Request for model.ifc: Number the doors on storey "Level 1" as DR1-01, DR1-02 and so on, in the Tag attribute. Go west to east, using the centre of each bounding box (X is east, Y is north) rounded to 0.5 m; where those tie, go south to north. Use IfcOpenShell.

First a look at what the model holds.

```python
import ifcopenshell
import ifcopenshell.util.element
import ifcopenshell.util.placement

model = ifcopenshell.open("model.ifc")
print(model.schema)
storey = next(s for s in model.by_type("IfcBuildingStorey") if s.Name == "Level 1")
doors = [e for e in ifcopenshell.util.element.get_decomposition(storey) if e.is_a("IfcDoor")]
for e in sorted(doors, key=lambda e: e.id()):
    origin = ifcopenshell.util.placement.get_local_placement(e.ObjectPlacement)[:3, 3]
    print(e.id(), e.Tag, e.Name, origin.round(2) + 0.0, sep=" | ")
```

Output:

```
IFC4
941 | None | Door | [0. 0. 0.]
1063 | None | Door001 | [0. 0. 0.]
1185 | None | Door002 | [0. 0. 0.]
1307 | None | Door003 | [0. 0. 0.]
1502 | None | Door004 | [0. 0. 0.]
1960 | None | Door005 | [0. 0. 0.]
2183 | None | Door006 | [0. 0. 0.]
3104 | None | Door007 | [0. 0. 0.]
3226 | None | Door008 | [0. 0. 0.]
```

```python
import ifcopenshell
import ifcopenshell.geom
import ifcopenshell.util.element
import ifcopenshell.util.shape

model = ifcopenshell.open("model.ifc")
settings = ifcopenshell.geom.settings()
settings.set("use-world-coords", True)


def centre(element):
    shape = ifcopenshell.geom.create_shape(settings, element)
    return ifcopenshell.util.shape.get_bbox_centroid(shape.geometry)


storey = next(s for s in model.by_type("IfcBuildingStorey") if s.Name == "Level 1")
doors = [e for e in ifcopenshell.util.element.get_decomposition(storey) if e.is_a("IfcDoor")]

# Insertion points can sit at a corner or the storey origin, so sort by the geometry (in metres).
centres = {e: centre(e) for e in doors}
doors.sort(key=lambda e: (round(centres[e][0] / 0.5), centres[e][1]))

for i, e in enumerate(doors, start=1):
    number = f"DR1-{i:02d}"
    e.Tag = number
    print(e.id(), number)

model.write("model-out.ifc")
```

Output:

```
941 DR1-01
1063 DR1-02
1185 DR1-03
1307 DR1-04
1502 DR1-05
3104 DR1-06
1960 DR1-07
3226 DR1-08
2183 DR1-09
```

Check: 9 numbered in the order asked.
